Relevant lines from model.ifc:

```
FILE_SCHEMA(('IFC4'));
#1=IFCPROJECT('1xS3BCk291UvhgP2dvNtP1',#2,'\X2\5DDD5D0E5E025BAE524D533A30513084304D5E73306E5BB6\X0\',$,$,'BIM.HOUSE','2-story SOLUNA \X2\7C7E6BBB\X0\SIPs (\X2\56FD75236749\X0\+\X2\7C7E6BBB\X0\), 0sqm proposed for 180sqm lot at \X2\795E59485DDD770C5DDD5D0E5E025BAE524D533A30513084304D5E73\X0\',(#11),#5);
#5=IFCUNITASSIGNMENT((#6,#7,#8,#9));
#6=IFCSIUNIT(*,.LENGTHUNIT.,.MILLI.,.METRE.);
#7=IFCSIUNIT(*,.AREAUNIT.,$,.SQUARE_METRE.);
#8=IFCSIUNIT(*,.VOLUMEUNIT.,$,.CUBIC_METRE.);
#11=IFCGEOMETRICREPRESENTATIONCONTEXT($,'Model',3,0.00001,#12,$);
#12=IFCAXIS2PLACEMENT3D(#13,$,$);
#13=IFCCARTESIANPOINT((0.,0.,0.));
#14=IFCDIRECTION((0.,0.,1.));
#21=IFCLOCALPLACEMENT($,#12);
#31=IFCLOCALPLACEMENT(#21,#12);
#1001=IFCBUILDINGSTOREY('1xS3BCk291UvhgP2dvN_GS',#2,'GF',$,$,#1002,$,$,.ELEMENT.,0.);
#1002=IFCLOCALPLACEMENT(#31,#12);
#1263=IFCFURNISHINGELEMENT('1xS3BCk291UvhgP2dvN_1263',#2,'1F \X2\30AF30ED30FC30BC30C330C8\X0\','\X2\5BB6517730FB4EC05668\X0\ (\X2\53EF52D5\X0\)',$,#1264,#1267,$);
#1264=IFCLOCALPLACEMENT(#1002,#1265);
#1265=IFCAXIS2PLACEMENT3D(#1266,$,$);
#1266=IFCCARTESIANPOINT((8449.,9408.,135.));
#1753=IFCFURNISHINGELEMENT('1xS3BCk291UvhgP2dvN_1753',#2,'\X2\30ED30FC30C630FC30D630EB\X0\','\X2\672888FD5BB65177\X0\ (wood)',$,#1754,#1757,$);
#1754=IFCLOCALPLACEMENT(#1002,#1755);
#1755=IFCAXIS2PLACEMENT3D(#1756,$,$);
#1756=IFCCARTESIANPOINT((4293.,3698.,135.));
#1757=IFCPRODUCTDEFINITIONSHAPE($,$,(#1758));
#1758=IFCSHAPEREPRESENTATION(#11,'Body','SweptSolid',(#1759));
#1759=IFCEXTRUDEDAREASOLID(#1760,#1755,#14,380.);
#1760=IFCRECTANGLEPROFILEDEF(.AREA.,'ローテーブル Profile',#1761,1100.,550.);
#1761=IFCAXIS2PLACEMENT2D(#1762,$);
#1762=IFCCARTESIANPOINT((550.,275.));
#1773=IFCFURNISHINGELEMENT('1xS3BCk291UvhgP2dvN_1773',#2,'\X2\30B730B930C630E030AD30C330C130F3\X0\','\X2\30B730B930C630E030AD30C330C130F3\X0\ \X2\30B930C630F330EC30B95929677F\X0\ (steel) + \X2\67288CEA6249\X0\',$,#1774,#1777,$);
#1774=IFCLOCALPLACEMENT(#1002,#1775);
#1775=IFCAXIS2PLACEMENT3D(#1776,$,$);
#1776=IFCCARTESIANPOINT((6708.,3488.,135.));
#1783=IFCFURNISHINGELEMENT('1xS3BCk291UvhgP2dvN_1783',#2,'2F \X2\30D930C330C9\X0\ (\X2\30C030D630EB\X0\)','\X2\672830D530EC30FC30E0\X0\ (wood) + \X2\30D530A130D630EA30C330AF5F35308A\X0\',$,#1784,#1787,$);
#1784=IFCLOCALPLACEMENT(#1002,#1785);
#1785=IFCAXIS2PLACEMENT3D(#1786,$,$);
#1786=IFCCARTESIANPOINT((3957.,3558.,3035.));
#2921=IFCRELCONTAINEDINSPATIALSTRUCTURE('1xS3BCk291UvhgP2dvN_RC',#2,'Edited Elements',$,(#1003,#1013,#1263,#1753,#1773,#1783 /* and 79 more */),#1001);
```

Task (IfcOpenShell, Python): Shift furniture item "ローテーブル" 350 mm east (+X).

```python
import ifcopenshell
import ifcopenshell.api.geometry
import ifcopenshell.util.placement
import ifcopenshell.util.unit

model = ifcopenshell.open("model.ifc")
unit_scale = ifcopenshell.util.unit.calculate_unit_scale(model)

item = model.by_guid("1xS3BCk291UvhgP2dvN_1753")
matrix = ifcopenshell.util.placement.get_local_placement(item.ObjectPlacement)
matrix[0, 3] += 0.35 / unit_scale
ifcopenshell.api.geometry.edit_object_placement(model, product=item, matrix=matrix, is_si=False)

print(ifcopenshell.util.placement.get_local_placement(item.ObjectPlacement).round(3) + 0.0)

model.write("model_rev.ifc")
```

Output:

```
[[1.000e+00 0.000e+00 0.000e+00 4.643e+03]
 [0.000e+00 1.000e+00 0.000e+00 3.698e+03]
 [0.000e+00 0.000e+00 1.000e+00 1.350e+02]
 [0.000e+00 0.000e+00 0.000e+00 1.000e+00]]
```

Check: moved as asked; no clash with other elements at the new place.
